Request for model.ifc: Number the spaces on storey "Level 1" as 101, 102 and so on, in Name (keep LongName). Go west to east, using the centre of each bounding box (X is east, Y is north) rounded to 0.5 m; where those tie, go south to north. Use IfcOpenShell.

First a look at what the model holds.

```python
import ifcopenshell
import ifcopenshell.util.element
import ifcopenshell.util.placement

model = ifcopenshell.open("model.ifc")
print(model.schema)
storey = next(s for s in model.by_type("IfcBuildingStorey") if s.Name == "Level 1")
spaces = [e for e in ifcopenshell.util.element.get_decomposition(storey) if e.is_a("IfcSpace")]
for e in sorted(spaces, key=lambda e: e.id()):
    origin = ifcopenshell.util.placement.get_local_placement(e.ObjectPlacement)[:3, 3]
    print(e.id(), e.Name, e.LongName, origin.round(2) + 0.0, sep=" | ")
```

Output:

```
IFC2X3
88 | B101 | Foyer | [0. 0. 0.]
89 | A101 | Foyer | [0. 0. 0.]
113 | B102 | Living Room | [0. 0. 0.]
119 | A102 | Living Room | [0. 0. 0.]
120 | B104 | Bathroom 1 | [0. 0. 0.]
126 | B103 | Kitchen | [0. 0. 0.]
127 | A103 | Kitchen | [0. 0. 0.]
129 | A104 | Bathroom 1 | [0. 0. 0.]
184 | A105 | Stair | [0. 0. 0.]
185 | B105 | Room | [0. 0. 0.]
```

```python
import ifcopenshell
import ifcopenshell.geom
import ifcopenshell.util.element
import ifcopenshell.util.shape

model = ifcopenshell.open("model.ifc")
settings = ifcopenshell.geom.settings()
settings.set("use-world-coords", True)


def centre(element):
    shape = ifcopenshell.geom.create_shape(settings, element)
    return ifcopenshell.util.shape.get_bbox_centroid(shape.geometry)


storey = next(s for s in model.by_type("IfcBuildingStorey") if s.Name == "Level 1")
spaces = [e for e in ifcopenshell.util.element.get_decomposition(storey) if e.is_a("IfcSpace")]

# Insertion points can sit at a corner or the storey origin, so sort by the geometry (in metres).
centres = {e: centre(e) for e in spaces}
spaces.sort(key=lambda e: (round(centres[e][0] / 0.5), centres[e][1]))

for i, e in enumerate(spaces, start=1):
    number = f"1{i:02d}"
    e.Name = number
    print(e.id(), number)

model.write("model_edited.ifc")
```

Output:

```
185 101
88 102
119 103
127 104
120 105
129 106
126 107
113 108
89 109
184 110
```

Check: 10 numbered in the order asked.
